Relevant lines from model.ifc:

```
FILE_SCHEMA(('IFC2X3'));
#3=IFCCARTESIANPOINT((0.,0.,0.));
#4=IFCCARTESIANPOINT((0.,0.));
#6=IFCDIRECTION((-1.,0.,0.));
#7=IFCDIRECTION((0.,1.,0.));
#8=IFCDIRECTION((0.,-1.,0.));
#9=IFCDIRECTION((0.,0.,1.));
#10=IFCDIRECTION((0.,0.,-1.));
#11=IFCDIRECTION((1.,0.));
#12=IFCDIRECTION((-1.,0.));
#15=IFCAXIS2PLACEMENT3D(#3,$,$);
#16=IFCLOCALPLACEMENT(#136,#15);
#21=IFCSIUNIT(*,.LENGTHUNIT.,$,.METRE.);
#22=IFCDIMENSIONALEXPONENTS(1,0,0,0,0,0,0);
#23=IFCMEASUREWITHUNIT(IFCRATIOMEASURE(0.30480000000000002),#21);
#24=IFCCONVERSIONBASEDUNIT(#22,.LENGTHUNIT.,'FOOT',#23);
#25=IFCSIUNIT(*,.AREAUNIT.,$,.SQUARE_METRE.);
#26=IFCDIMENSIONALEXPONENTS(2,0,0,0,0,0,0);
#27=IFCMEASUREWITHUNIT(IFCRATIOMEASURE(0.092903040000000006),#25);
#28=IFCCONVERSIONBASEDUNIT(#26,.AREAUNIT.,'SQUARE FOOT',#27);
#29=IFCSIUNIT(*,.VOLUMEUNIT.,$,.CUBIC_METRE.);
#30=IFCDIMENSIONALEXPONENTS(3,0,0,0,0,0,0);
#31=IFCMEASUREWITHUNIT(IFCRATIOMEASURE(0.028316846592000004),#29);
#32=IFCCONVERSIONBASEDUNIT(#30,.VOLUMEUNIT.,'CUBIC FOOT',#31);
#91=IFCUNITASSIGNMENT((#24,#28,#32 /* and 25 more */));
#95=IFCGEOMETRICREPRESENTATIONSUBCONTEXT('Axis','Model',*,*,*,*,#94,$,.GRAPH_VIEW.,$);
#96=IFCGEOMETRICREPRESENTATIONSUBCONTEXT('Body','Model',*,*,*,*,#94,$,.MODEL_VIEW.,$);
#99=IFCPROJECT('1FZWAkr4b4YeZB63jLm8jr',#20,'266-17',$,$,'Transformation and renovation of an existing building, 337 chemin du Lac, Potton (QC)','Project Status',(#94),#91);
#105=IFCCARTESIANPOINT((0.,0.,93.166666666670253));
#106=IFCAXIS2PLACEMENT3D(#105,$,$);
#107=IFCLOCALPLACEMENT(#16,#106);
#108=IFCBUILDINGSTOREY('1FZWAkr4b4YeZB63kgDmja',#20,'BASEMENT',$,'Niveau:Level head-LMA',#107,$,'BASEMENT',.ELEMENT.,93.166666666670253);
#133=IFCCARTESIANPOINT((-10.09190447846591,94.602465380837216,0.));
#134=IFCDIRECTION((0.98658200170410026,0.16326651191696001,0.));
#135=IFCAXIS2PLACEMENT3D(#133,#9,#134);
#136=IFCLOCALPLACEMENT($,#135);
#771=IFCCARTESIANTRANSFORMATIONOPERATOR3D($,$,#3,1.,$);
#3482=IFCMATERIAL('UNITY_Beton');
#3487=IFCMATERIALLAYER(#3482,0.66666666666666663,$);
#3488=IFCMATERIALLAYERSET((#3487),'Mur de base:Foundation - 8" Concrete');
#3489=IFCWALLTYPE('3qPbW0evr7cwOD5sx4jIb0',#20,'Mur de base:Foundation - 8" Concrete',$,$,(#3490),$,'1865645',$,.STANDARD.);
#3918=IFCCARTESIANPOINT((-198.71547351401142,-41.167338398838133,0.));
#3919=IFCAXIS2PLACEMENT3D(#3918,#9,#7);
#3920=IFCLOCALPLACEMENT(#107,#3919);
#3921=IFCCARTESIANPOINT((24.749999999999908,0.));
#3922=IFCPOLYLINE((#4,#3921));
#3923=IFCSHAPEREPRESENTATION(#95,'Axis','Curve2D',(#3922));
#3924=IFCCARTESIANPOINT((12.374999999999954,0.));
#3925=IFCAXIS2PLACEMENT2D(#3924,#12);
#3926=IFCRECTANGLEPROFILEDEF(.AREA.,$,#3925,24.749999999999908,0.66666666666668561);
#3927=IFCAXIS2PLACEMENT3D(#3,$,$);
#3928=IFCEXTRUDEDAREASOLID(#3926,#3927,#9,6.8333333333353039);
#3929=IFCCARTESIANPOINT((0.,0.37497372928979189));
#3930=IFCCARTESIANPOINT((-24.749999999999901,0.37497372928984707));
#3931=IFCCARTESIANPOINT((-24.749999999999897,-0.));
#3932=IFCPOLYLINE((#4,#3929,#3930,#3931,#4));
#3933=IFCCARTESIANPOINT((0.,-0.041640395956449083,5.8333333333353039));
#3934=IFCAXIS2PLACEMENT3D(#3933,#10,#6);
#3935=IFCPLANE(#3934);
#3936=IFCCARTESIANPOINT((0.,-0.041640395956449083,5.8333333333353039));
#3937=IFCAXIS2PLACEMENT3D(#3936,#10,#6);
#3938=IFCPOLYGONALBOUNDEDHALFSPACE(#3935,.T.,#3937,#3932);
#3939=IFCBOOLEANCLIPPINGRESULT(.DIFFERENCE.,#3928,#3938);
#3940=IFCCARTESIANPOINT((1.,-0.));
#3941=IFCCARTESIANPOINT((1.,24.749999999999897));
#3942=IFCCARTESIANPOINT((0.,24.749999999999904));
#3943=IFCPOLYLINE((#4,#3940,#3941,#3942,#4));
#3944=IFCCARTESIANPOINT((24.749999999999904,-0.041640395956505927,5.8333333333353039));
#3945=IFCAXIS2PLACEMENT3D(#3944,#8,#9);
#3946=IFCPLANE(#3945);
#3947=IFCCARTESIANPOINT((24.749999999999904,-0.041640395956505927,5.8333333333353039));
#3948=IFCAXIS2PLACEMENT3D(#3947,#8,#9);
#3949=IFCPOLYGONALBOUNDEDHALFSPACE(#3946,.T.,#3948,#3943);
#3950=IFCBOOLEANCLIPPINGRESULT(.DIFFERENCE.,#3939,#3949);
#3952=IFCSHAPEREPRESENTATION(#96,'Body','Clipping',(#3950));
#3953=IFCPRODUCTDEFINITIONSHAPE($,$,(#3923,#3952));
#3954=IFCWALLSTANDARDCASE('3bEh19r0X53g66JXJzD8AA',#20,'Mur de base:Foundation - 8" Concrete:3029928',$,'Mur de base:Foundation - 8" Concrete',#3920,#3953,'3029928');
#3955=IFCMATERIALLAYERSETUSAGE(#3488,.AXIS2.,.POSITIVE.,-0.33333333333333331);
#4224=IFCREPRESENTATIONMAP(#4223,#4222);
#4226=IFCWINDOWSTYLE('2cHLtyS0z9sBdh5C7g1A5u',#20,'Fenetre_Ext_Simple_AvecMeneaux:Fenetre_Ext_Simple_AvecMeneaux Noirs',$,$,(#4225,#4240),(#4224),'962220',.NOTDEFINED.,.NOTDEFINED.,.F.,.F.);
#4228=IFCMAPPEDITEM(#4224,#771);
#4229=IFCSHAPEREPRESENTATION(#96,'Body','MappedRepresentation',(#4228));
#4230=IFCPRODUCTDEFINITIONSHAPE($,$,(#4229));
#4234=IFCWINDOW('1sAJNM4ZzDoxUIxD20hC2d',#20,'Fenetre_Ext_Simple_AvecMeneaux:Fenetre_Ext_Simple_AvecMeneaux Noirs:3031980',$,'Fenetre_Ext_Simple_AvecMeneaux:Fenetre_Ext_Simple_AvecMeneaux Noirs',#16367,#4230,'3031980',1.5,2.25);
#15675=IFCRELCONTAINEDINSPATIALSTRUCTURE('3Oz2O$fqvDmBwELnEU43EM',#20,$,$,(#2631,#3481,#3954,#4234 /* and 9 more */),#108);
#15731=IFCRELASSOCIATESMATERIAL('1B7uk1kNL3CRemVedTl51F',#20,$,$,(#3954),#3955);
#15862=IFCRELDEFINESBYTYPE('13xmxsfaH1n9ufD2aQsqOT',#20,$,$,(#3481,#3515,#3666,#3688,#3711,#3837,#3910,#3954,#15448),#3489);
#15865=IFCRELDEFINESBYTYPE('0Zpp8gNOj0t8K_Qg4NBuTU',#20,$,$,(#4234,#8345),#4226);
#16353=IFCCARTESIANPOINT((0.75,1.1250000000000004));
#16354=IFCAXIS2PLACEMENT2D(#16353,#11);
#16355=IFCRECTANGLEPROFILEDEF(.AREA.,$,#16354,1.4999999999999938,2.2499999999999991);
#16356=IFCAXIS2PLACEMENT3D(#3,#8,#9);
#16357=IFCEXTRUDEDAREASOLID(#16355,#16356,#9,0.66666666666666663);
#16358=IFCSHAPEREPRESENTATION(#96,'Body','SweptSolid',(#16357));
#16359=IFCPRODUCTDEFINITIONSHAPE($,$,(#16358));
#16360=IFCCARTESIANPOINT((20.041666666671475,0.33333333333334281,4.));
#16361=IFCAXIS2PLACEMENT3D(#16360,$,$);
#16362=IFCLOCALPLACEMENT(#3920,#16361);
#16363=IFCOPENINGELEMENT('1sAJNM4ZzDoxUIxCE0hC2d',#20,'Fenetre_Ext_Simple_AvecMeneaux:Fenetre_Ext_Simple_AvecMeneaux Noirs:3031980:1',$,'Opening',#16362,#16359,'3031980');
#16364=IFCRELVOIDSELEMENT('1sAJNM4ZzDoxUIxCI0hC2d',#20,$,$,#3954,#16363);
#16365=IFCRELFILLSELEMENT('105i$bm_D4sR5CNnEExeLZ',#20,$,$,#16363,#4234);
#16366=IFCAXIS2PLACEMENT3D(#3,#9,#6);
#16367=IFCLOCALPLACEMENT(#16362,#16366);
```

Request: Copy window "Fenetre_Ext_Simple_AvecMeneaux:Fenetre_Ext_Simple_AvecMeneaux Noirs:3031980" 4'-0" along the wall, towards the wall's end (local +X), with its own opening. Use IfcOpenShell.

```python
import ifcopenshell
import ifcopenshell.api.feature
import ifcopenshell.api.geometry
import ifcopenshell.api.root
import ifcopenshell.geom
import ifcopenshell.util.element
import ifcopenshell.util.placement
import ifcopenshell.util.shape
import ifcopenshell.util.unit

model = ifcopenshell.open("model.ifc")
unit_scale = ifcopenshell.util.unit.calculate_unit_scale(model)
settings = ifcopenshell.geom.settings()


def volume(element):
    """Net volume in cubic metres, openings subtracted."""
    shape = ifcopenshell.geom.create_shape(settings, element)
    return ifcopenshell.util.shape.get_volume(shape.geometry)


def reuse_history(source, copy):
    """copy_class also copies each property set's owner history, people and application; keep the originals."""
    for rel in copy.IsDefinedBy:
        if rel.is_a("IfcRelDefinesByProperties") and (history := rel.RelatingPropertyDefinition.OwnerHistory):
            rel.RelatingPropertyDefinition.OwnerHistory = source.OwnerHistory
            ifcopenshell.util.element.remove_deep2(model, history)


window = model.by_guid("1sAJNM4ZzDoxUIxD20hC2d")
opening = window.FillsVoids[0].RelatingOpeningElement
wall = opening.VoidsElements[0].RelatingBuildingElement
before = volume(wall)
shift = ifcopenshell.util.placement.get_local_placement(wall.ObjectPlacement)[:3, 0] * 48 * 0.0254 / unit_scale

# copy_class copies the void relationship, type, container and properties, but no geometry.
new_opening = ifcopenshell.api.root.copy_class(model, product=opening)
new_opening.Representation = ifcopenshell.util.element.copy_deep(
    model, opening.Representation, exclude=["IfcGeometricRepresentationContext", "IfcRepresentationMap"]
)
new_opening.Name = "Fenetre_Ext_Simple_AvecMeneaux:Fenetre_Ext_Simple_AvecMeneaux Noirs"
new_opening.Tag = None
new_window = ifcopenshell.api.root.copy_class(model, product=window)
new_window.Representation = ifcopenshell.util.element.copy_deep(
    model, window.Representation, exclude=["IfcGeometricRepresentationContext", "IfcRepresentationMap"]
)
new_window.Name = "Fenetre_Ext_Simple_AvecMeneaux:Fenetre_Ext_Simple_AvecMeneaux Noirs"
new_window.Tag = None
reuse_history(window, new_window)
fills = ifcopenshell.api.feature.add_filling(model, opening=new_opening, element=new_window)
fills.OwnerHistory = new_window.OwnerHistory  # required in IFC2X3

for old, new in ((opening, new_opening), (window, new_window)):
    matrix = ifcopenshell.util.placement.get_local_placement(old.ObjectPlacement)
    matrix[:3, 3] += shift
    ifcopenshell.api.geometry.edit_object_placement(model, product=new, matrix=matrix, is_si=False)

after = volume(wall)

print(f"wall volume {before:.3f} -> {after:.3f} m3")

model.write("model_edited.ifc")
```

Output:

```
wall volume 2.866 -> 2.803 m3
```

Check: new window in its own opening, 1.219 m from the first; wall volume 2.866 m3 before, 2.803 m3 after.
